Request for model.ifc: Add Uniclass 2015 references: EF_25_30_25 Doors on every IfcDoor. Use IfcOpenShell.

First a look at what the model holds.

```python
import ifcopenshell

model = ifcopenshell.open("model.ifc")
print(model.schema)
print("classifications:", [c.Name for c in model.by_type("IfcClassification")])
for ifc_class in ("IfcDoor", "IfcRoof", "IfcStair", "IfcWall", "IfcWindow"):
    print(ifc_class, len(model.by_type(ifc_class)))
```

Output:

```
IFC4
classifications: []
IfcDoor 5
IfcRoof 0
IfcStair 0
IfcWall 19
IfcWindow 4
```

```python
import ifcopenshell
import ifcopenshell.api.classification

model = ifcopenshell.open("model.ifc")

system = ifcopenshell.api.classification.add_classification(model, classification="Uniclass 2015")

codes = {
    "IfcDoor": ("EF_25_30_25", "Doors"),
}
for ifc_class, (code, name) in codes.items():
    products = model.by_type(ifc_class)
    ifcopenshell.api.classification.add_reference(
        model, products=products, classification=system, identification=code, name=name
    )
    print(code, len(products))

model.write("model_updated.ifc")
```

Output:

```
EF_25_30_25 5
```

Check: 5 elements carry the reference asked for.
